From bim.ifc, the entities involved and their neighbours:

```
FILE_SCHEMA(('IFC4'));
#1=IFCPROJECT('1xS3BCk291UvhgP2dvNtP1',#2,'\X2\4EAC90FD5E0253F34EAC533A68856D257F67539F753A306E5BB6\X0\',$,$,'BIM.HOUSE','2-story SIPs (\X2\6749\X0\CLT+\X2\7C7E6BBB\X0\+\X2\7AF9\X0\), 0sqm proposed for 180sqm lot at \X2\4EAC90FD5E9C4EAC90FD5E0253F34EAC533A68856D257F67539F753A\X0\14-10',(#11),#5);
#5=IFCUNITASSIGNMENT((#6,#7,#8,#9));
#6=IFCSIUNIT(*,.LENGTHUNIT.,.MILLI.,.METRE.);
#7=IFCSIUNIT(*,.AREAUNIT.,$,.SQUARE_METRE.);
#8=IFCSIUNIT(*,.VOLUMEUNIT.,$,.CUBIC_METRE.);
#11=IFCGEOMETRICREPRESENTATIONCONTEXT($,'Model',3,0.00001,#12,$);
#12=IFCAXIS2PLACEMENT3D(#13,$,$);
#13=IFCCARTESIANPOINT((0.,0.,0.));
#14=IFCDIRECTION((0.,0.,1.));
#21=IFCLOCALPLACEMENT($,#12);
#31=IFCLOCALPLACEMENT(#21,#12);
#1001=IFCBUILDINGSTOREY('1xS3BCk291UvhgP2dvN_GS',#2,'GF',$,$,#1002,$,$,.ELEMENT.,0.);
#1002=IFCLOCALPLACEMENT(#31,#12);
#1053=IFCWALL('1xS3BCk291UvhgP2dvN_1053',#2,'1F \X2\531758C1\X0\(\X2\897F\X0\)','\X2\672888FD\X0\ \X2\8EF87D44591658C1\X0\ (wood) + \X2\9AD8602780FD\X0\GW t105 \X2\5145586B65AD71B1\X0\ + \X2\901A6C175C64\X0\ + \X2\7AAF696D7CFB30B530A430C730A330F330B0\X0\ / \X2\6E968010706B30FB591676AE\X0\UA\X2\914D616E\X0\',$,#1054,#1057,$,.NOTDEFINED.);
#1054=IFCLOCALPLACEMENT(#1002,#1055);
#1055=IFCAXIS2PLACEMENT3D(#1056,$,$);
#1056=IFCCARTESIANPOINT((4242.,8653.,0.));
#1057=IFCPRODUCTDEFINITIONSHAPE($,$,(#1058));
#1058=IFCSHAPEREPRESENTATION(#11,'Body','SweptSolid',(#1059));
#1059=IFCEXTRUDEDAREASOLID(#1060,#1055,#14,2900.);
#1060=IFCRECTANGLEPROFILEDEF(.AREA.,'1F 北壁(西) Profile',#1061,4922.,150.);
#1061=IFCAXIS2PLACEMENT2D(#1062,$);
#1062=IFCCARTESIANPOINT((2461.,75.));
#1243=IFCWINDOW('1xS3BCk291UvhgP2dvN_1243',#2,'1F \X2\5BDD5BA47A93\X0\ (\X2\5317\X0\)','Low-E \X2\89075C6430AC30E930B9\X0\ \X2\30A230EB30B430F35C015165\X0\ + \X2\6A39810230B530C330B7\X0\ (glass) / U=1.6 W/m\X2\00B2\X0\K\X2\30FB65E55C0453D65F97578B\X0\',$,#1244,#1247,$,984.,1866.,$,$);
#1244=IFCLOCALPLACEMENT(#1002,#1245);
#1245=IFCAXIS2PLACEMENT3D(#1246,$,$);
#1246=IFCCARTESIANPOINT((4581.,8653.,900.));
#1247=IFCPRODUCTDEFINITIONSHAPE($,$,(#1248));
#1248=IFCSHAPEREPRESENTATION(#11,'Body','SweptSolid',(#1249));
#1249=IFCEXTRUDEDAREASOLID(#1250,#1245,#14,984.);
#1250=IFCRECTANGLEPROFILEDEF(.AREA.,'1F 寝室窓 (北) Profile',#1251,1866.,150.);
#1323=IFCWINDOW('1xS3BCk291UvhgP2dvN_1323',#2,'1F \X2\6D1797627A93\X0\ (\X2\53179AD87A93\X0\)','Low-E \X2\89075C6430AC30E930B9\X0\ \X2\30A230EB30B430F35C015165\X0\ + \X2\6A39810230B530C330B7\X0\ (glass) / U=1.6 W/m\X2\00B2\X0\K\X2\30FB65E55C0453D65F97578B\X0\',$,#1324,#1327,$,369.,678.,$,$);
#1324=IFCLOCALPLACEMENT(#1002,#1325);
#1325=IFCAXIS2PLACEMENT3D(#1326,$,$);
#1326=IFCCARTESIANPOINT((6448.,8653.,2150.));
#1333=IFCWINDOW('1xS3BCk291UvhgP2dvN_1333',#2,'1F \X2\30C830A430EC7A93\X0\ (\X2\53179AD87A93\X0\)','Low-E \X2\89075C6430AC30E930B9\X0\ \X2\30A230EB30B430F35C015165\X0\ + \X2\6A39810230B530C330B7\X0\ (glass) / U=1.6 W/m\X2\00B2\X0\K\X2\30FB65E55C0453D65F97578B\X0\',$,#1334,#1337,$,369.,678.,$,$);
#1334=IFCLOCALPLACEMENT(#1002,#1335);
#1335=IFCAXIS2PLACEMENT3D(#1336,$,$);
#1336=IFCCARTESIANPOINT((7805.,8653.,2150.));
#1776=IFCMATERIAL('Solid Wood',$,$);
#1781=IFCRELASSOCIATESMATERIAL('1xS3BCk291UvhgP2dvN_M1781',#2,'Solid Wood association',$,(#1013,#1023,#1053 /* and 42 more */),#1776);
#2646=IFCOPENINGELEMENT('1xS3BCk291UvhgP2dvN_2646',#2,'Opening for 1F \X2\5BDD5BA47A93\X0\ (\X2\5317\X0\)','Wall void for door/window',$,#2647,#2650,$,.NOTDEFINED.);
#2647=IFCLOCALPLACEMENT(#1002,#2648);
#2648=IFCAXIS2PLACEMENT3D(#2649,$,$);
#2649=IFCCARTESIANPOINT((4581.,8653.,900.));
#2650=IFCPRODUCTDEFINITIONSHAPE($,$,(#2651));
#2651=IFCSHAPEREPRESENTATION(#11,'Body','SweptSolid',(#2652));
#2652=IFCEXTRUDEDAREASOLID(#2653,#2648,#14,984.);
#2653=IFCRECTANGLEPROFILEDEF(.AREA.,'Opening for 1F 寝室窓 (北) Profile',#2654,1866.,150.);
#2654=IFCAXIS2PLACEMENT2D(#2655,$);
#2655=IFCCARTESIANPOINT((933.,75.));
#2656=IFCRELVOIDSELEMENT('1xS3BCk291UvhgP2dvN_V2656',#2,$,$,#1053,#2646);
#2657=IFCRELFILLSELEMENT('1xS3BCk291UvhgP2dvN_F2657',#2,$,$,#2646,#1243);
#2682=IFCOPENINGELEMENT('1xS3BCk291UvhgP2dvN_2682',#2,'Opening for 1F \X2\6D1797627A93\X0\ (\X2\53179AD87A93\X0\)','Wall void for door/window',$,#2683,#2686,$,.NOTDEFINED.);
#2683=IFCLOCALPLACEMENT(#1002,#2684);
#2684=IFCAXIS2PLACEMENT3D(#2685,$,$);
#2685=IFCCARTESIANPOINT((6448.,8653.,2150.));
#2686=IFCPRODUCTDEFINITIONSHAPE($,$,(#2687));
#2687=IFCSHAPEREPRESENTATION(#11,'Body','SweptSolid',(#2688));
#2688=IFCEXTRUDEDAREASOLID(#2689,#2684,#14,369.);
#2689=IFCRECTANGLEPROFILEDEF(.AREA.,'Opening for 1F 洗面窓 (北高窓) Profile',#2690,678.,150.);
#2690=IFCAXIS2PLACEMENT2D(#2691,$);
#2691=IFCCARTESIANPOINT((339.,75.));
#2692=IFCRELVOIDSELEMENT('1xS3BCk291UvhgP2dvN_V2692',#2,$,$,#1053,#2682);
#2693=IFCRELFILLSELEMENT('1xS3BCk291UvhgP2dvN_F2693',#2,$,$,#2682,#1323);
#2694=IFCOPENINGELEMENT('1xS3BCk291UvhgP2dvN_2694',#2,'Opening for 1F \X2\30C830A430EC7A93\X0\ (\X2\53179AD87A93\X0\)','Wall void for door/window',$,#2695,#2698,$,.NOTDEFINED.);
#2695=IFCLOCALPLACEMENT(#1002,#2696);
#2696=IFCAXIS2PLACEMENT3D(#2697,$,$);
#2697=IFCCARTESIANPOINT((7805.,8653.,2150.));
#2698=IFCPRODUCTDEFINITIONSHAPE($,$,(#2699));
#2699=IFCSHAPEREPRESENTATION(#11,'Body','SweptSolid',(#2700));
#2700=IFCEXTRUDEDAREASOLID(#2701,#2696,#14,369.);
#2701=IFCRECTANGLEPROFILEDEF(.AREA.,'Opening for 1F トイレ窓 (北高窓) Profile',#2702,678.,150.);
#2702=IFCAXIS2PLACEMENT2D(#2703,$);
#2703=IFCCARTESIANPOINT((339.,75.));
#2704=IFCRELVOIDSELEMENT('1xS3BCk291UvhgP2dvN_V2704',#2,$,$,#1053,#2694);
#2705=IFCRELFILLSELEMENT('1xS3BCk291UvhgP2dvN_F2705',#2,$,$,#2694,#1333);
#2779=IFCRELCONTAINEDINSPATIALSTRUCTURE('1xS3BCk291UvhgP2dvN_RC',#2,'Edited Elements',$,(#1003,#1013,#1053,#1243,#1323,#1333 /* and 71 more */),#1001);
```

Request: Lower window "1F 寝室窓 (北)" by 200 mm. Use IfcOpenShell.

```python
import numpy as np
import ifcopenshell
import ifcopenshell.api.geometry
import ifcopenshell.util.placement
import ifcopenshell.util.unit

model = ifcopenshell.open("bim.ifc")
unit_scale = ifcopenshell.util.unit.calculate_unit_scale(model)

window = model.by_guid("1xS3BCk291UvhgP2dvN_1243")
opening = window.FillsVoids[0].RelatingOpeningElement
dz = -200.0

shift = np.array([0.0, 0.0, dz])
# The window is not placed relative to its opening, so move both.
for product in (opening, window):
    matrix = ifcopenshell.util.placement.get_local_placement(product.ObjectPlacement)
    matrix[:3, 3] += shift
    ifcopenshell.api.geometry.edit_object_placement(model, product=product, matrix=matrix, is_si=False)

print(f"moved by {dz * unit_scale:+.3f} m")

model.write("bim_rev.ifc")
```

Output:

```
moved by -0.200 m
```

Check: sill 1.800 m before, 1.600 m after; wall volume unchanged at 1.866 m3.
